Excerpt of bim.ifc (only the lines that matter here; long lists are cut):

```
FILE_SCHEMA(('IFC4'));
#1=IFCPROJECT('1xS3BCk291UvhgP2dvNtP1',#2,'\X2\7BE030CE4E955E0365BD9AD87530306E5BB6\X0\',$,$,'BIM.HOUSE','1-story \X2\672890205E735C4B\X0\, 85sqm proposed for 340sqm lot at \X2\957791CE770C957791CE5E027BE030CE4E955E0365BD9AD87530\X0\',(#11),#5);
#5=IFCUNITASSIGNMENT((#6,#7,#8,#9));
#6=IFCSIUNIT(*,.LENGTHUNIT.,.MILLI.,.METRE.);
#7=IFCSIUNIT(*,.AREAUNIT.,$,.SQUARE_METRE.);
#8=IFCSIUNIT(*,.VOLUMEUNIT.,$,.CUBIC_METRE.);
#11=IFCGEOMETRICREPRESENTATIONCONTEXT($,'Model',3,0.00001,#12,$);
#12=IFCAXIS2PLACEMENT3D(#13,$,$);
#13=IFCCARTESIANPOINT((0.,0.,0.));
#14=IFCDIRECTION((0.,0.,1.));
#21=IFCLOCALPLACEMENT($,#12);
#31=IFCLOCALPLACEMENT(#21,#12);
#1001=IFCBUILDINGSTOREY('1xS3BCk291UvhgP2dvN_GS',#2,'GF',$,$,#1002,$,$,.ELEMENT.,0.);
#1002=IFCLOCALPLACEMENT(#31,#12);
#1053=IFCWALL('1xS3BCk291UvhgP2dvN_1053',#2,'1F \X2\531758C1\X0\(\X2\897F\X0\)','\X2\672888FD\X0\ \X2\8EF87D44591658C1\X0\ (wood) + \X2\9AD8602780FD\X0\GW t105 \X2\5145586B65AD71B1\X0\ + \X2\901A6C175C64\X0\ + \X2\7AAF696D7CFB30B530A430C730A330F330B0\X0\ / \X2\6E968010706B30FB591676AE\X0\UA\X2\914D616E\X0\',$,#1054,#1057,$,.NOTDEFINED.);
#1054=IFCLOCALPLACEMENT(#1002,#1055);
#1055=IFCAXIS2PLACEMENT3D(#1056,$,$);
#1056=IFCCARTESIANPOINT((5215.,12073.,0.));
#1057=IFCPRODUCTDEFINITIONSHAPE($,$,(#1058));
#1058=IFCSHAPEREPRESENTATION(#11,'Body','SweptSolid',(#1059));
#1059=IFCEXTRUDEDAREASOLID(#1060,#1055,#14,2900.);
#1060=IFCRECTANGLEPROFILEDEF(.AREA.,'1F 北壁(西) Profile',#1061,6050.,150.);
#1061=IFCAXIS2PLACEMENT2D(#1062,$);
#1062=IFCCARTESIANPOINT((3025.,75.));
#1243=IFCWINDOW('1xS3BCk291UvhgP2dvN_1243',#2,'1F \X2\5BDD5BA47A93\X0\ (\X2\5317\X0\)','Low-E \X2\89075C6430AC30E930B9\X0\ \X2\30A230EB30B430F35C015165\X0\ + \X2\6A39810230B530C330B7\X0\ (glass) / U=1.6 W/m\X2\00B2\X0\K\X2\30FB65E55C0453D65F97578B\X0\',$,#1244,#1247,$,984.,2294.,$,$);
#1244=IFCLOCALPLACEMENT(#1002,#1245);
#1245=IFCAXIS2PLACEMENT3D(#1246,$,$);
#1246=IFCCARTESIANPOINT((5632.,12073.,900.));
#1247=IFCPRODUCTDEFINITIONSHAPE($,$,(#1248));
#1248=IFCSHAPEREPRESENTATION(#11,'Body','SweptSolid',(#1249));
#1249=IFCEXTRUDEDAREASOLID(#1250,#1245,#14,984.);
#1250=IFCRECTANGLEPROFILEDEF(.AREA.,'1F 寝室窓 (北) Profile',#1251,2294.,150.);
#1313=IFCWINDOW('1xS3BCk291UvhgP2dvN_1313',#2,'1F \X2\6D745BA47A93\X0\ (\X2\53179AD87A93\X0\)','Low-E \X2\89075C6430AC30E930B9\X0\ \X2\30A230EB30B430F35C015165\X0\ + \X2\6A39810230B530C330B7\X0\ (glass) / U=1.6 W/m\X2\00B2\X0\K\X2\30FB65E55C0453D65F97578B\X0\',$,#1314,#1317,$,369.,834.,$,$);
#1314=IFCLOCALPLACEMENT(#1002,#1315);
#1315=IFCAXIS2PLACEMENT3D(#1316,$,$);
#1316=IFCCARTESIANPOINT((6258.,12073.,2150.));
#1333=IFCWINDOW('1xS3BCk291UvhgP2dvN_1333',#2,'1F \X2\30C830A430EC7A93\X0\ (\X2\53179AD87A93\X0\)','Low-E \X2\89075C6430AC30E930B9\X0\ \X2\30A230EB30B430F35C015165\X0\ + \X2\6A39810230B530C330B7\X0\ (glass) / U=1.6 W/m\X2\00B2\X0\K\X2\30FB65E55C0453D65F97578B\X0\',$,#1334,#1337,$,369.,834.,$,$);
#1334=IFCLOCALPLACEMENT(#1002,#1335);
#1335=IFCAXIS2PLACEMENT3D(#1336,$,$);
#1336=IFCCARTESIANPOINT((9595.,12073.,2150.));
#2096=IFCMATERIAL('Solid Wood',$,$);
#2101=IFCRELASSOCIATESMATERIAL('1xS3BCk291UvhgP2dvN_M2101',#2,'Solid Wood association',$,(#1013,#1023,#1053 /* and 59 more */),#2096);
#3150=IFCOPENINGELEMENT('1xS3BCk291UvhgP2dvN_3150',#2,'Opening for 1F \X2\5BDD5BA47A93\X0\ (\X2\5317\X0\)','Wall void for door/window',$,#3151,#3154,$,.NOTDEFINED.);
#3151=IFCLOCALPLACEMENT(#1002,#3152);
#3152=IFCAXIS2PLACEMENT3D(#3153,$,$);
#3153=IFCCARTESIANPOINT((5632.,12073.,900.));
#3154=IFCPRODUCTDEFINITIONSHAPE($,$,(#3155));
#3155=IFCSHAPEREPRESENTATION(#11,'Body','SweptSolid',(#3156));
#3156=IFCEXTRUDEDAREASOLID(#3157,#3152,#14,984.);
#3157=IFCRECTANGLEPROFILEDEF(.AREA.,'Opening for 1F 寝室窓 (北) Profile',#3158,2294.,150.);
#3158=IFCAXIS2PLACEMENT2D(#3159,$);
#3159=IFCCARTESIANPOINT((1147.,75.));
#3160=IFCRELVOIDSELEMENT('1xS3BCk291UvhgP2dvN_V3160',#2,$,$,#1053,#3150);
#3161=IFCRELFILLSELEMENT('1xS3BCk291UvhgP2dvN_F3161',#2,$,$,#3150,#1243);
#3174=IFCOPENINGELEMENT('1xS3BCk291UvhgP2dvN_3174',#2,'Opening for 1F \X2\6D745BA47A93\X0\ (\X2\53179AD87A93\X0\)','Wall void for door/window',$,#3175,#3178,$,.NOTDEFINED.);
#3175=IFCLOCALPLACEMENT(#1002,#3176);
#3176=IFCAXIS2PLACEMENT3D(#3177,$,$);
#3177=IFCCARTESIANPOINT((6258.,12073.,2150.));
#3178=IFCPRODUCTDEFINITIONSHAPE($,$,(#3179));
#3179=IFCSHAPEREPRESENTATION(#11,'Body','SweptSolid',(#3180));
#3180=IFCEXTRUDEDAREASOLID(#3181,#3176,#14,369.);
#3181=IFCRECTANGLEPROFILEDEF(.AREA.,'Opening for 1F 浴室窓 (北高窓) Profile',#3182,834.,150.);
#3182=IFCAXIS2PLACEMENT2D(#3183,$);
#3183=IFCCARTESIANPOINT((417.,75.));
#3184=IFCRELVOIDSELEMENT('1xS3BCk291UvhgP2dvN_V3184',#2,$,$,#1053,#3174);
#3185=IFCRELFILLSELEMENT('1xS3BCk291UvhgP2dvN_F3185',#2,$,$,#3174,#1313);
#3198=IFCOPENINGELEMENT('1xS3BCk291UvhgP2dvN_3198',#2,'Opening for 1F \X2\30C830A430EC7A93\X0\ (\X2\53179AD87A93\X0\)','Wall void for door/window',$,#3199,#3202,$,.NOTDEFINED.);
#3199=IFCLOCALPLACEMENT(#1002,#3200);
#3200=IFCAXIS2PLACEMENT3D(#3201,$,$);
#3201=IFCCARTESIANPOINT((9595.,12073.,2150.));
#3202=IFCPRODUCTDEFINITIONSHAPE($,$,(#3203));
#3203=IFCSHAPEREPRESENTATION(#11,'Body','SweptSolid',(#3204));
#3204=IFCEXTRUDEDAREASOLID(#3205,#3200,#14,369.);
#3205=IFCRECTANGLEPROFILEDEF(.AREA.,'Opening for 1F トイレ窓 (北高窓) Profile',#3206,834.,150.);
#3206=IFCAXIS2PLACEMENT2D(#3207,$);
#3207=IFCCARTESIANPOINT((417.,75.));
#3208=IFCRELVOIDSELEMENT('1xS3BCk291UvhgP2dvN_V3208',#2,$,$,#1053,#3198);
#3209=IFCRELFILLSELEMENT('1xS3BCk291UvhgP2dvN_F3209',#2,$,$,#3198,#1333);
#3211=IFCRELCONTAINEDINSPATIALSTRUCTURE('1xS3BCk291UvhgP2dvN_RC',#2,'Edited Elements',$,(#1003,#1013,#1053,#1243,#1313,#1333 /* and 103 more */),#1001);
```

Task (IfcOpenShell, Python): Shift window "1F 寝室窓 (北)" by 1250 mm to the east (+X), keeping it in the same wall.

```python
import ifcopenshell
import ifcopenshell.api.geometry
import ifcopenshell.util.placement

model = ifcopenshell.open("bim.ifc")

window = model.by_guid("1xS3BCk291UvhgP2dvN_1243")
opening = window.FillsVoids[0].RelatingOpeningElement
wall = opening.VoidsElements[0].RelatingBuildingElement

wall_matrix = ifcopenshell.util.placement.get_local_placement(wall.ObjectPlacement)
shift = wall_matrix[:3, 0] * 1250.0
before = ifcopenshell.util.placement.get_local_placement(window.ObjectPlacement)[:3, 3].copy()

# The window is not placed relative to its opening, so move both.
for product in (opening, window):
    matrix = ifcopenshell.util.placement.get_local_placement(product.ObjectPlacement)
    matrix[:3, 3] += shift
    ifcopenshell.api.geometry.edit_object_placement(model, product=product, matrix=matrix, is_si=False)

after = ifcopenshell.util.placement.get_local_placement(window.ObjectPlacement)[:3, 3]
print("window moved by", (after - before).round(3) + 0.0)

model.write("bim_rev.ifc")
```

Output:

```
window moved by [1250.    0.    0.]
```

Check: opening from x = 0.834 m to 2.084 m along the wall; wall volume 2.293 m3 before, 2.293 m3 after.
